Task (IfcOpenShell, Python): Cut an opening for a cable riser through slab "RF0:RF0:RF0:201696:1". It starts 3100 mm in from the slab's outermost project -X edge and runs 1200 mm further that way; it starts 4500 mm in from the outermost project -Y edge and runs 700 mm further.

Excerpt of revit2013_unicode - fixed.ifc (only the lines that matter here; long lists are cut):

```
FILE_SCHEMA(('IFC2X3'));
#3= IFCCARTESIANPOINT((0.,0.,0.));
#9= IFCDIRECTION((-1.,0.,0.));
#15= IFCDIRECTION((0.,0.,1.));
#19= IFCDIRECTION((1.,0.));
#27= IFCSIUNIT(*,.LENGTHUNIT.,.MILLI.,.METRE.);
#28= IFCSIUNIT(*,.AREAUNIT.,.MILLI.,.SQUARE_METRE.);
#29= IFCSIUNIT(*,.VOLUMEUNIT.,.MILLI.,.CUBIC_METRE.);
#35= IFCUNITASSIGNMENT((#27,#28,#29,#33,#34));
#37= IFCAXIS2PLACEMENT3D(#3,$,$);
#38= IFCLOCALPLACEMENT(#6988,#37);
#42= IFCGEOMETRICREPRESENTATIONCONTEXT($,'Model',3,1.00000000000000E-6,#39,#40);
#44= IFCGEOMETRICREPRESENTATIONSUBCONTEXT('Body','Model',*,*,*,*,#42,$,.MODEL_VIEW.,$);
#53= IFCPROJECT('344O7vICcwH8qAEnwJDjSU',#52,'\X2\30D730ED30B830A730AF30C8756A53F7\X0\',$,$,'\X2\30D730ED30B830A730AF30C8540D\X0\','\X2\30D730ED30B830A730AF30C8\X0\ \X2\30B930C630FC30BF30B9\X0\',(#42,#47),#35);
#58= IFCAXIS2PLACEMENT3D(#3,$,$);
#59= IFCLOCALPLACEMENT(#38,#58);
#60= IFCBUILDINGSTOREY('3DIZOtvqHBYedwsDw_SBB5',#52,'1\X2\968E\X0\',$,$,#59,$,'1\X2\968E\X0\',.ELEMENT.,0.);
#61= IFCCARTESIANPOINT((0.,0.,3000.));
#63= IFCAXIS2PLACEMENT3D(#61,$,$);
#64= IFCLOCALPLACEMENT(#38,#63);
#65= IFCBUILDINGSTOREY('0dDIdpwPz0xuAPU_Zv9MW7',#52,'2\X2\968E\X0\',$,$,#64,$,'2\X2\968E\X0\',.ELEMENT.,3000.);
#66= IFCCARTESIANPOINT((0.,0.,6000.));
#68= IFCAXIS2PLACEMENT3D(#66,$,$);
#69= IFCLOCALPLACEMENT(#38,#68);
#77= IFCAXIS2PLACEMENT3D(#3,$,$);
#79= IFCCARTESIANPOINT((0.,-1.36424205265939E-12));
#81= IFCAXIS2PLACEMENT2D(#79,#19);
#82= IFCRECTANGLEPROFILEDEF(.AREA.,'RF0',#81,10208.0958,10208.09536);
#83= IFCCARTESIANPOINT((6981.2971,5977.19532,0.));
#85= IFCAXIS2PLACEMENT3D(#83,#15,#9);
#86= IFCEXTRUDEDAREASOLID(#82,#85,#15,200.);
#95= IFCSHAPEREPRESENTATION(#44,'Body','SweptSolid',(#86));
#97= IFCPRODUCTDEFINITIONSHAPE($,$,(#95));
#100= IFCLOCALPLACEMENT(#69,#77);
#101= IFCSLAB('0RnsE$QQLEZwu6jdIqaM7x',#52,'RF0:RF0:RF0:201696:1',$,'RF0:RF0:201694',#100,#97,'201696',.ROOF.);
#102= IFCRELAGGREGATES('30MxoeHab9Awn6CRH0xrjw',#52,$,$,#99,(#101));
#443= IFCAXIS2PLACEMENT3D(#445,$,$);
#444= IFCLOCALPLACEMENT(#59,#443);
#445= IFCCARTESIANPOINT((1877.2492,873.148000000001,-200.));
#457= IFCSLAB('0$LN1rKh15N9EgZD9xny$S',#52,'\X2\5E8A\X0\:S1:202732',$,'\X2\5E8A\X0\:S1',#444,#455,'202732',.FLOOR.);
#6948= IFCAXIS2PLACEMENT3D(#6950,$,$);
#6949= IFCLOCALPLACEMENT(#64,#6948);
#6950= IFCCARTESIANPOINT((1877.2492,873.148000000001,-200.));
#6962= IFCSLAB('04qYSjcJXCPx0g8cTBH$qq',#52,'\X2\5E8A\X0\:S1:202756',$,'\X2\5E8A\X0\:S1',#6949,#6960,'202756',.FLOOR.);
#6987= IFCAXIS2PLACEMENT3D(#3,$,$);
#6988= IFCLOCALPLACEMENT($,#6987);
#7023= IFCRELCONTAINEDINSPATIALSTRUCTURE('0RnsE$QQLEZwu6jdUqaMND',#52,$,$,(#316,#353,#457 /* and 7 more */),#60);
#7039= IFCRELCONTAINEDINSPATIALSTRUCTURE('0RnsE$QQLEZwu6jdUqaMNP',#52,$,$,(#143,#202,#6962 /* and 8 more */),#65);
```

```python
import numpy as np
import ifcopenshell
import ifcopenshell.api.feature
import ifcopenshell.api.geometry
import ifcopenshell.api.root
import ifcopenshell.geom
import ifcopenshell.util.placement
import ifcopenshell.util.representation
import ifcopenshell.util.shape
import ifcopenshell.util.unit

model = ifcopenshell.open("revit2013_unicode - fixed.ifc")
unit_scale = ifcopenshell.util.unit.calculate_unit_scale(model)
settings = ifcopenshell.geom.settings()


def volume(element):
    """Net volume in cubic metres, openings subtracted."""
    shape = ifcopenshell.geom.create_shape(settings, element)
    return ifcopenshell.util.shape.get_volume(shape.geometry)


slab = model.by_id(101)
before = volume(slab)

# Extent in the slab's own axes, in metres. The edges named are its -X and -Y sides.
slab_shape = ifcopenshell.geom.create_shape(settings, slab)
vertices = ifcopenshell.util.shape.get_vertices(slab_shape.geometry)
x_min, y_min, bottom = vertices.min(axis=0)
top = vertices[:, 2].max()

opening = ifcopenshell.api.root.create_entity(model, ifc_class="IfcOpeningElement", name="Cable riser opening")
context = ifcopenshell.util.representation.get_context(model, "Model", "Body", "MODEL_VIEW")
width, depth = 1.2, 0.7
outline = [(0.0, 0.0), (width, 0.0), (width, depth), (0.0, depth), (0.0, 0.0)]
# Overshoot both faces by 50 mm so the cut is clean.
shape = ifcopenshell.api.geometry.add_slab_representation(
    model, context=context, depth=top - bottom + 0.1, polyline=outline
)
ifcopenshell.api.geometry.assign_representation(model, product=opening, representation=shape)

matrix = ifcopenshell.util.placement.get_local_placement(slab.ObjectPlacement)
matrix[:, 3] = matrix @ np.append(np.array([x_min + 3.1, y_min + 4.5, bottom - 0.05]) / unit_scale, 1.0)
ifcopenshell.api.geometry.edit_object_placement(model, product=opening, matrix=matrix, is_si=False)
ifcopenshell.api.feature.add_feature(model, feature=opening, element=slab)

after = volume(slab)

print(f"slab volume {before:.3f} -> {after:.3f} m3")

model.write("revit2013_unicode - fixed_updated.ifc")
```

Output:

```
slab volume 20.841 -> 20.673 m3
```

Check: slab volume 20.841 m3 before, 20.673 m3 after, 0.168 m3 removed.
